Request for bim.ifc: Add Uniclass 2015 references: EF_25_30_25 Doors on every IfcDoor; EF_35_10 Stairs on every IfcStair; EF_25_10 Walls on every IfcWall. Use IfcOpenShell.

First a look at what the model holds.

```python
import ifcopenshell

model = ifcopenshell.open("bim.ifc")
print(model.schema)
print("classifications:", [c.Name for c in model.by_type("IfcClassification")])
for ifc_class in ("IfcDoor", "IfcRoof", "IfcStair", "IfcWall", "IfcWindow"):
    print(ifc_class, len(model.by_type(ifc_class)))
```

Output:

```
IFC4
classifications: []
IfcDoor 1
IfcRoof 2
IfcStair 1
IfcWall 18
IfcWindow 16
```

```python
import ifcopenshell
import ifcopenshell.api.classification

model = ifcopenshell.open("bim.ifc")

system = ifcopenshell.api.classification.add_classification(model, classification="Uniclass 2015")

codes = {
    "IfcDoor": ("EF_25_30_25", "Doors"),
    "IfcStair": ("EF_35_10", "Stairs"),
    "IfcWall": ("EF_25_10", "Walls"),
}
for ifc_class, (code, name) in codes.items():
    products = model.by_type(ifc_class)
    ifcopenshell.api.classification.add_reference(
        model, products=products, classification=system, identification=code, name=name
    )
    print(code, len(products))

model.write("bim_edited.ifc")
```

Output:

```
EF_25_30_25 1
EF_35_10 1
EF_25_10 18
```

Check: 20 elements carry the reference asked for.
